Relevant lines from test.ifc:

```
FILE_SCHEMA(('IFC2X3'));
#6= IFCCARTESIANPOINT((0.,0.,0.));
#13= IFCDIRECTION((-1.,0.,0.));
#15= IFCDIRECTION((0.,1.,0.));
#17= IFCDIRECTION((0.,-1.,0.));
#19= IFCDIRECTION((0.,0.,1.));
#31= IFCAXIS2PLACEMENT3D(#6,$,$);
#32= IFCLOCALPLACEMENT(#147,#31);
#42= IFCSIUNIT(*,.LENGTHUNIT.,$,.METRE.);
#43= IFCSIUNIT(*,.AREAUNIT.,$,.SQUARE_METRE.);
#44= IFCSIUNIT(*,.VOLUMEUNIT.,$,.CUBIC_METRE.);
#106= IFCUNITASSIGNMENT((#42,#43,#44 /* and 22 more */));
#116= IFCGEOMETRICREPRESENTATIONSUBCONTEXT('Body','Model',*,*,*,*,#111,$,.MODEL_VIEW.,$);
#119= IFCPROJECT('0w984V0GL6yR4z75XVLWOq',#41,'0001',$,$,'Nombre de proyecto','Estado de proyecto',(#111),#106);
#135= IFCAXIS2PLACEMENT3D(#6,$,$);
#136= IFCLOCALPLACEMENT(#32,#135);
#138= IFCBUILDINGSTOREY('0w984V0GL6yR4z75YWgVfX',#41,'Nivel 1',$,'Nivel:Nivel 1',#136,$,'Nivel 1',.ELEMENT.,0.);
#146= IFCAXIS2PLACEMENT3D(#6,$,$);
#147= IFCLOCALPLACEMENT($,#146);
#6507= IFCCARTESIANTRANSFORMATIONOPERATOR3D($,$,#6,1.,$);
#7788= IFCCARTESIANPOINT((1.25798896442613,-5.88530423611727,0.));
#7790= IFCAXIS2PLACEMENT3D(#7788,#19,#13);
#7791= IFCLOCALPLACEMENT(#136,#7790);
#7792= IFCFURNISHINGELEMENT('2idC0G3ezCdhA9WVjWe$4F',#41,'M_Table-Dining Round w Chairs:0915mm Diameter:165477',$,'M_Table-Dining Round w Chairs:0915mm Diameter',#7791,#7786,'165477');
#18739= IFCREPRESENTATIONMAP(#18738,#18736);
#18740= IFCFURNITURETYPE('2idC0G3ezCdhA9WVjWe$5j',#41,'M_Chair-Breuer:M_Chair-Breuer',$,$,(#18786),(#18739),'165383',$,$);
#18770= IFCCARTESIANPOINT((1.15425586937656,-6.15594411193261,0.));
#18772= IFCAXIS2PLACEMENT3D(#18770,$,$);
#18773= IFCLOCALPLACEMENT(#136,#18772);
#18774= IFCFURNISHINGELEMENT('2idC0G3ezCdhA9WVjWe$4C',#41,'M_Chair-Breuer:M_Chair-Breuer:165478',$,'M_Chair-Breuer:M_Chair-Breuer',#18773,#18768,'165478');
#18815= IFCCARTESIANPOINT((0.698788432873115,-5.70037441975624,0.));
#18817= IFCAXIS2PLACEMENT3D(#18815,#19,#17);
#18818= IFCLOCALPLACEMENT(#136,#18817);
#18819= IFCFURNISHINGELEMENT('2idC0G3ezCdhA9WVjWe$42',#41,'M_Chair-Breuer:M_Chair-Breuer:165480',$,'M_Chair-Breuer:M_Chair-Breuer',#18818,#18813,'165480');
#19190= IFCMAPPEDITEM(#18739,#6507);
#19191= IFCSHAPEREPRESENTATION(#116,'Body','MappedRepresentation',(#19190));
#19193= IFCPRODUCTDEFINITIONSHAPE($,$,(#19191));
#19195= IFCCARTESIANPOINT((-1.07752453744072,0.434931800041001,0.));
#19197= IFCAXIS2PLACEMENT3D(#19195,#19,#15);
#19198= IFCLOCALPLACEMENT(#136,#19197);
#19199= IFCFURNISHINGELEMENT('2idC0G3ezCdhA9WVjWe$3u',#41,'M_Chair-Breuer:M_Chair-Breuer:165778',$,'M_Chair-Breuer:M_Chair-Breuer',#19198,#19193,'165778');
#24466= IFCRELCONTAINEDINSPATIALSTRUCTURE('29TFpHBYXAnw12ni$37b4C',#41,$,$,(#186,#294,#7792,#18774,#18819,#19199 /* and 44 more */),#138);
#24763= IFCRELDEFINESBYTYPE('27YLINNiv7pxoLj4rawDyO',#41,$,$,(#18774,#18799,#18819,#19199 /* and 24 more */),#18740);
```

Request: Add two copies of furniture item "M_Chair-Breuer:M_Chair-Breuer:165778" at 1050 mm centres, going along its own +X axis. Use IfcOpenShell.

```python
import ifcopenshell
import ifcopenshell.api.geometry
import ifcopenshell.api.root
import ifcopenshell.util.element
import ifcopenshell.util.placement

model = ifcopenshell.open("test.ifc")


def reuse_history(source, copy):
    """copy_class also copies each property set's owner history, people and application; keep the originals."""
    for rel in copy.IsDefinedBy:
        if rel.is_a("IfcRelDefinesByProperties") and (history := rel.RelatingPropertyDefinition.OwnerHistory):
            rel.RelatingPropertyDefinition.OwnerHistory = source.OwnerHistory
            ifcopenshell.util.element.remove_deep2(model, history)


source = model.by_guid("2idC0G3ezCdhA9WVjWe$3u")
base = ifcopenshell.util.placement.get_local_placement(source.ObjectPlacement)
step = base[:3, 0] * 1.05

for i in range(1, 3):
    copy = ifcopenshell.api.root.copy_class(model, product=source)
    copy.Representation = ifcopenshell.util.element.copy_deep(
        model, source.Representation, exclude=["IfcGeometricRepresentationContext", "IfcRepresentationMap"]
    )
    copy.Name = "M_Chair-Breuer:M_Chair-Breuer"
    copy.Tag = None
    reuse_history(source, copy)
    matrix = base.copy()
    matrix[:3, 3] += i * step
    print("added at", matrix[:3, 3].round(3) + 0.0)
    ifcopenshell.api.geometry.edit_object_placement(model, product=copy, matrix=matrix, is_si=False)

model.write("test_edited.ifc")
```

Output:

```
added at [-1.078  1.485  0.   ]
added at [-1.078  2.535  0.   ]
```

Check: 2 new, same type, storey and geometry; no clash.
